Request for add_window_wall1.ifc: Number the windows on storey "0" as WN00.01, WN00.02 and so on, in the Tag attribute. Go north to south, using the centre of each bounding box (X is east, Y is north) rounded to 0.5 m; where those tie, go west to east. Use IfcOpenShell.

First a look at what the model holds.

```python
import ifcopenshell
import ifcopenshell.util.element
import ifcopenshell.util.placement

model = ifcopenshell.open("add_window_wall1.ifc")
print(model.schema)
storey = next(s for s in model.by_type("IfcBuildingStorey") if s.Name == "0")
windows = [e for e in ifcopenshell.util.element.get_decomposition(storey) if e.is_a("IfcWindow")]
for e in sorted(windows, key=lambda e: e.id()):
    origin = ifcopenshell.util.placement.get_local_placement(e.ObjectPlacement)[:3, 3]
    print(e.id(), e.Tag, e.Name, origin.round(2) + 0.0, sep=" | ")
```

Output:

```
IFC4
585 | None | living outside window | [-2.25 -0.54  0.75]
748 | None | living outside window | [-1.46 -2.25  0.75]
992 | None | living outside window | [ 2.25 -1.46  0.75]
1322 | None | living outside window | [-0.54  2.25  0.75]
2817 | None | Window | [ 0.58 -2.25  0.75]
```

```python
import ifcopenshell
import ifcopenshell.geom
import ifcopenshell.util.element
import ifcopenshell.util.shape

model = ifcopenshell.open("add_window_wall1.ifc")
settings = ifcopenshell.geom.settings()
settings.set("use-world-coords", True)


def centre(element):
    shape = ifcopenshell.geom.create_shape(settings, element)
    return ifcopenshell.util.shape.get_bbox_centroid(shape.geometry)


storey = next(s for s in model.by_type("IfcBuildingStorey") if s.Name == "0")
windows = [e for e in ifcopenshell.util.element.get_decomposition(storey) if e.is_a("IfcWindow")]

# Insertion points can sit at a corner or the storey origin, so sort by the geometry (in metres).
centres = {e: centre(e) for e in windows}
windows.sort(key=lambda e: (-round(centres[e][1] / 0.5), centres[e][0]))

for i, e in enumerate(windows, start=1):
    number = f"WN00.{i:02d}"
    e.Tag = number
    print(e.id(), number)

model.write("add_window_wall1_edited.ifc")
```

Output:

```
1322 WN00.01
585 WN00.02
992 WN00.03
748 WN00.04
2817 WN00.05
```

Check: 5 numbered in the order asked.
